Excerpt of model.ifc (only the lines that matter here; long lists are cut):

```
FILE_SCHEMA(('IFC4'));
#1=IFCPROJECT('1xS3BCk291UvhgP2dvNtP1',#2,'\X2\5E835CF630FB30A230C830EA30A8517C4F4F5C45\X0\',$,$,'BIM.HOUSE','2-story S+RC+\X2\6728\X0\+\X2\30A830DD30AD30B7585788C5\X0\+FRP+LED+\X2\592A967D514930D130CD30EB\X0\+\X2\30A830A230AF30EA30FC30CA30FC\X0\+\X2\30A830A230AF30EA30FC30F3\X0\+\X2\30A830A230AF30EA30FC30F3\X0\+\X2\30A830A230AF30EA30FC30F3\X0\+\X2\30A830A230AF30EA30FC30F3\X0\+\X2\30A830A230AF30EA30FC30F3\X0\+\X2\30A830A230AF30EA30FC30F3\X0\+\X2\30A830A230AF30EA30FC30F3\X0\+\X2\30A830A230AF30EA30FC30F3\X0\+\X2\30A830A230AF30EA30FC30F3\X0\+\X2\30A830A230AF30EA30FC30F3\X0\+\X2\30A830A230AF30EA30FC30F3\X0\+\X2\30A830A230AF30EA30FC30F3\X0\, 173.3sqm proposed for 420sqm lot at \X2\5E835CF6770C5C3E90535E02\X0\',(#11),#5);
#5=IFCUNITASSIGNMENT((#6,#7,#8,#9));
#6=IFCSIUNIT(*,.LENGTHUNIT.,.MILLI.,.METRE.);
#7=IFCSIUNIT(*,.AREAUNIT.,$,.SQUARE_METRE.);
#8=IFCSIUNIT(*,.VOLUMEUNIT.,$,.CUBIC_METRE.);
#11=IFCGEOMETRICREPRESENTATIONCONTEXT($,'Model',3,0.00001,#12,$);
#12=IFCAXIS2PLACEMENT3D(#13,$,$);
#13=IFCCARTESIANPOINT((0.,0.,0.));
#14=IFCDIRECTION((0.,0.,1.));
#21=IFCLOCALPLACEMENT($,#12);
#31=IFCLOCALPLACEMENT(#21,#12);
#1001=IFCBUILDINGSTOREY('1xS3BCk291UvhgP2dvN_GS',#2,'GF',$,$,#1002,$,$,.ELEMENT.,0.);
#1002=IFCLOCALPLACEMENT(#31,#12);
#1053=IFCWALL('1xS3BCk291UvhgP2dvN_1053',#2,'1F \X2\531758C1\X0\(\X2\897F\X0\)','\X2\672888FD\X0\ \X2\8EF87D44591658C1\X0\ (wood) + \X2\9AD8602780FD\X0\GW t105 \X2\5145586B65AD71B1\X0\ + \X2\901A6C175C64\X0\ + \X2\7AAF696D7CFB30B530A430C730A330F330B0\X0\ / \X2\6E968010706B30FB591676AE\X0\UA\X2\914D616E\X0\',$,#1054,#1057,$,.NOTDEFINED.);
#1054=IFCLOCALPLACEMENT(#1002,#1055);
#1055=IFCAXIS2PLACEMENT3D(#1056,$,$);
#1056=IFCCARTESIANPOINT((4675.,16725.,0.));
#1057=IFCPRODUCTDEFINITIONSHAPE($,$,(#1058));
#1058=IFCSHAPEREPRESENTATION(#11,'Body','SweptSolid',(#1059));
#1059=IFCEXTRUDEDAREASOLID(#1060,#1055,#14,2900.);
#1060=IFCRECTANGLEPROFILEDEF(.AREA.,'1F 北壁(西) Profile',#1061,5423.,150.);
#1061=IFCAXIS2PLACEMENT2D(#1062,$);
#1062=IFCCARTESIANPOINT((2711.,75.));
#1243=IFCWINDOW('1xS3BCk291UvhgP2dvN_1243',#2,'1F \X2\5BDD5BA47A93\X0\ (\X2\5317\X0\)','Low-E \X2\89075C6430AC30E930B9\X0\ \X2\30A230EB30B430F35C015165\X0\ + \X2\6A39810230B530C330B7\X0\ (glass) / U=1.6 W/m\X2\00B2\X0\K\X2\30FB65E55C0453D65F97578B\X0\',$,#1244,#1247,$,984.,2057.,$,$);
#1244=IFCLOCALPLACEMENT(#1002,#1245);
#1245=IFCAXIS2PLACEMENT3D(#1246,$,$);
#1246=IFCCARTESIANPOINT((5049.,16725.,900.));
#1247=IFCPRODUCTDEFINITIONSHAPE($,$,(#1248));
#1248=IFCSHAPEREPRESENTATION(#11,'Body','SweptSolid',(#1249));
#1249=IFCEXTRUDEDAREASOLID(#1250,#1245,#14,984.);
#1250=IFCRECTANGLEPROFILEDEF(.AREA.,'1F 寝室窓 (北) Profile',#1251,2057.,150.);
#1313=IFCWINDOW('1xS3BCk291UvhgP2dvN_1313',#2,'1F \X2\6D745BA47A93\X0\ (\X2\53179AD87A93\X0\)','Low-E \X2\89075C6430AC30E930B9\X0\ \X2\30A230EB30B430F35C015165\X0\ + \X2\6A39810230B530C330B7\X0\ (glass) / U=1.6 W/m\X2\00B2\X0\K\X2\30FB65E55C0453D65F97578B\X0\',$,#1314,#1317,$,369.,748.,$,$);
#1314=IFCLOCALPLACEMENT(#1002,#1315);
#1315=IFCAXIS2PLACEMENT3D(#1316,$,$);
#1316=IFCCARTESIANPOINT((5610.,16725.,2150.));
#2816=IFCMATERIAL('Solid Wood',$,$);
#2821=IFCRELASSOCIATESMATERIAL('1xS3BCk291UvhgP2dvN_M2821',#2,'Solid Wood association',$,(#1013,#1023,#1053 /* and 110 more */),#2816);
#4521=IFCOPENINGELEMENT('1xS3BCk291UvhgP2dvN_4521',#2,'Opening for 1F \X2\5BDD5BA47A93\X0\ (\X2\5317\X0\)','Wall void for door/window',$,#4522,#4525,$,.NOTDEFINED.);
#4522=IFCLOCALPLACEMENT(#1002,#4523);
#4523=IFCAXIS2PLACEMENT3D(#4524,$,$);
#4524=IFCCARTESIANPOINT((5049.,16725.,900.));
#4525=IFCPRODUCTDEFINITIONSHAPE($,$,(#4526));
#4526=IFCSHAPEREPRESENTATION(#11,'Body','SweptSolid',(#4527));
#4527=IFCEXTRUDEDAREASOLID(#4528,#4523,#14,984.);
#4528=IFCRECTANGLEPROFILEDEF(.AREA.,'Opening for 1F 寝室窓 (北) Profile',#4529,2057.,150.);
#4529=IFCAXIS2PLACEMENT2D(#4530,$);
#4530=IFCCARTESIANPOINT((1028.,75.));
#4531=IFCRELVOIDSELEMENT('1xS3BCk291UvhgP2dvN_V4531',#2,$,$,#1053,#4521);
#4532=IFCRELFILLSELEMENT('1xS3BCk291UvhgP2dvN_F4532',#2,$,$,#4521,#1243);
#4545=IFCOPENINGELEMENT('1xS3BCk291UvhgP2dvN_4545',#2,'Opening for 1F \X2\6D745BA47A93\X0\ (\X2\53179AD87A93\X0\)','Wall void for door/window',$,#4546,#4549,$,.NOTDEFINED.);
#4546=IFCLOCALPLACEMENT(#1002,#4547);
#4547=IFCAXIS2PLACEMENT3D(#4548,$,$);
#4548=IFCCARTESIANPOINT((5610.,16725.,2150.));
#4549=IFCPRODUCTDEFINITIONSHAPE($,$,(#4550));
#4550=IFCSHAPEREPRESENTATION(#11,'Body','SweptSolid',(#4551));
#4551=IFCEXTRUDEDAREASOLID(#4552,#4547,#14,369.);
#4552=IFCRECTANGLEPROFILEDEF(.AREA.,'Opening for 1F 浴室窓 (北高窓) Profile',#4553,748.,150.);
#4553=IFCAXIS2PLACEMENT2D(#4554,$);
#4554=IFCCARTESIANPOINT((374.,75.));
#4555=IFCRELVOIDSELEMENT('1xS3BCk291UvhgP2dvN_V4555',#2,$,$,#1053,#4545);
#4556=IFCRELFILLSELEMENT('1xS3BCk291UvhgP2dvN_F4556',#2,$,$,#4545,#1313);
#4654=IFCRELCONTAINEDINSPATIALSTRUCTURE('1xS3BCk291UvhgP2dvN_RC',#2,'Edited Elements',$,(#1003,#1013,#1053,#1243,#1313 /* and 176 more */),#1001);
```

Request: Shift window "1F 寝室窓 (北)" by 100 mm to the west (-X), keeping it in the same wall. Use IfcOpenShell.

```python
import ifcopenshell
import ifcopenshell.api.geometry
import ifcopenshell.util.placement

model = ifcopenshell.open("model.ifc")

window = model.by_id(1243)
opening = window.FillsVoids[0].RelatingOpeningElement
wall = opening.VoidsElements[0].RelatingBuildingElement

wall_matrix = ifcopenshell.util.placement.get_local_placement(wall.ObjectPlacement)
shift = wall_matrix[:3, 0] * -100.0
before = ifcopenshell.util.placement.get_local_placement(window.ObjectPlacement)[:3, 3].copy()

# The window is not placed relative to its opening, so move both.
for product in (opening, window):
    matrix = ifcopenshell.util.placement.get_local_placement(product.ObjectPlacement)
    matrix[:3, 3] += shift
    ifcopenshell.api.geometry.edit_object_placement(model, product=product, matrix=matrix, is_si=False)

after = ifcopenshell.util.placement.get_local_placement(window.ObjectPlacement)[:3, 3]
print("window moved by", (after - before).round(3) + 0.0)

model.write("model-out.ifc")
```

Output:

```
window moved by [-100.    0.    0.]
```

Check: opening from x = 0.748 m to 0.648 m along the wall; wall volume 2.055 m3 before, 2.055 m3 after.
